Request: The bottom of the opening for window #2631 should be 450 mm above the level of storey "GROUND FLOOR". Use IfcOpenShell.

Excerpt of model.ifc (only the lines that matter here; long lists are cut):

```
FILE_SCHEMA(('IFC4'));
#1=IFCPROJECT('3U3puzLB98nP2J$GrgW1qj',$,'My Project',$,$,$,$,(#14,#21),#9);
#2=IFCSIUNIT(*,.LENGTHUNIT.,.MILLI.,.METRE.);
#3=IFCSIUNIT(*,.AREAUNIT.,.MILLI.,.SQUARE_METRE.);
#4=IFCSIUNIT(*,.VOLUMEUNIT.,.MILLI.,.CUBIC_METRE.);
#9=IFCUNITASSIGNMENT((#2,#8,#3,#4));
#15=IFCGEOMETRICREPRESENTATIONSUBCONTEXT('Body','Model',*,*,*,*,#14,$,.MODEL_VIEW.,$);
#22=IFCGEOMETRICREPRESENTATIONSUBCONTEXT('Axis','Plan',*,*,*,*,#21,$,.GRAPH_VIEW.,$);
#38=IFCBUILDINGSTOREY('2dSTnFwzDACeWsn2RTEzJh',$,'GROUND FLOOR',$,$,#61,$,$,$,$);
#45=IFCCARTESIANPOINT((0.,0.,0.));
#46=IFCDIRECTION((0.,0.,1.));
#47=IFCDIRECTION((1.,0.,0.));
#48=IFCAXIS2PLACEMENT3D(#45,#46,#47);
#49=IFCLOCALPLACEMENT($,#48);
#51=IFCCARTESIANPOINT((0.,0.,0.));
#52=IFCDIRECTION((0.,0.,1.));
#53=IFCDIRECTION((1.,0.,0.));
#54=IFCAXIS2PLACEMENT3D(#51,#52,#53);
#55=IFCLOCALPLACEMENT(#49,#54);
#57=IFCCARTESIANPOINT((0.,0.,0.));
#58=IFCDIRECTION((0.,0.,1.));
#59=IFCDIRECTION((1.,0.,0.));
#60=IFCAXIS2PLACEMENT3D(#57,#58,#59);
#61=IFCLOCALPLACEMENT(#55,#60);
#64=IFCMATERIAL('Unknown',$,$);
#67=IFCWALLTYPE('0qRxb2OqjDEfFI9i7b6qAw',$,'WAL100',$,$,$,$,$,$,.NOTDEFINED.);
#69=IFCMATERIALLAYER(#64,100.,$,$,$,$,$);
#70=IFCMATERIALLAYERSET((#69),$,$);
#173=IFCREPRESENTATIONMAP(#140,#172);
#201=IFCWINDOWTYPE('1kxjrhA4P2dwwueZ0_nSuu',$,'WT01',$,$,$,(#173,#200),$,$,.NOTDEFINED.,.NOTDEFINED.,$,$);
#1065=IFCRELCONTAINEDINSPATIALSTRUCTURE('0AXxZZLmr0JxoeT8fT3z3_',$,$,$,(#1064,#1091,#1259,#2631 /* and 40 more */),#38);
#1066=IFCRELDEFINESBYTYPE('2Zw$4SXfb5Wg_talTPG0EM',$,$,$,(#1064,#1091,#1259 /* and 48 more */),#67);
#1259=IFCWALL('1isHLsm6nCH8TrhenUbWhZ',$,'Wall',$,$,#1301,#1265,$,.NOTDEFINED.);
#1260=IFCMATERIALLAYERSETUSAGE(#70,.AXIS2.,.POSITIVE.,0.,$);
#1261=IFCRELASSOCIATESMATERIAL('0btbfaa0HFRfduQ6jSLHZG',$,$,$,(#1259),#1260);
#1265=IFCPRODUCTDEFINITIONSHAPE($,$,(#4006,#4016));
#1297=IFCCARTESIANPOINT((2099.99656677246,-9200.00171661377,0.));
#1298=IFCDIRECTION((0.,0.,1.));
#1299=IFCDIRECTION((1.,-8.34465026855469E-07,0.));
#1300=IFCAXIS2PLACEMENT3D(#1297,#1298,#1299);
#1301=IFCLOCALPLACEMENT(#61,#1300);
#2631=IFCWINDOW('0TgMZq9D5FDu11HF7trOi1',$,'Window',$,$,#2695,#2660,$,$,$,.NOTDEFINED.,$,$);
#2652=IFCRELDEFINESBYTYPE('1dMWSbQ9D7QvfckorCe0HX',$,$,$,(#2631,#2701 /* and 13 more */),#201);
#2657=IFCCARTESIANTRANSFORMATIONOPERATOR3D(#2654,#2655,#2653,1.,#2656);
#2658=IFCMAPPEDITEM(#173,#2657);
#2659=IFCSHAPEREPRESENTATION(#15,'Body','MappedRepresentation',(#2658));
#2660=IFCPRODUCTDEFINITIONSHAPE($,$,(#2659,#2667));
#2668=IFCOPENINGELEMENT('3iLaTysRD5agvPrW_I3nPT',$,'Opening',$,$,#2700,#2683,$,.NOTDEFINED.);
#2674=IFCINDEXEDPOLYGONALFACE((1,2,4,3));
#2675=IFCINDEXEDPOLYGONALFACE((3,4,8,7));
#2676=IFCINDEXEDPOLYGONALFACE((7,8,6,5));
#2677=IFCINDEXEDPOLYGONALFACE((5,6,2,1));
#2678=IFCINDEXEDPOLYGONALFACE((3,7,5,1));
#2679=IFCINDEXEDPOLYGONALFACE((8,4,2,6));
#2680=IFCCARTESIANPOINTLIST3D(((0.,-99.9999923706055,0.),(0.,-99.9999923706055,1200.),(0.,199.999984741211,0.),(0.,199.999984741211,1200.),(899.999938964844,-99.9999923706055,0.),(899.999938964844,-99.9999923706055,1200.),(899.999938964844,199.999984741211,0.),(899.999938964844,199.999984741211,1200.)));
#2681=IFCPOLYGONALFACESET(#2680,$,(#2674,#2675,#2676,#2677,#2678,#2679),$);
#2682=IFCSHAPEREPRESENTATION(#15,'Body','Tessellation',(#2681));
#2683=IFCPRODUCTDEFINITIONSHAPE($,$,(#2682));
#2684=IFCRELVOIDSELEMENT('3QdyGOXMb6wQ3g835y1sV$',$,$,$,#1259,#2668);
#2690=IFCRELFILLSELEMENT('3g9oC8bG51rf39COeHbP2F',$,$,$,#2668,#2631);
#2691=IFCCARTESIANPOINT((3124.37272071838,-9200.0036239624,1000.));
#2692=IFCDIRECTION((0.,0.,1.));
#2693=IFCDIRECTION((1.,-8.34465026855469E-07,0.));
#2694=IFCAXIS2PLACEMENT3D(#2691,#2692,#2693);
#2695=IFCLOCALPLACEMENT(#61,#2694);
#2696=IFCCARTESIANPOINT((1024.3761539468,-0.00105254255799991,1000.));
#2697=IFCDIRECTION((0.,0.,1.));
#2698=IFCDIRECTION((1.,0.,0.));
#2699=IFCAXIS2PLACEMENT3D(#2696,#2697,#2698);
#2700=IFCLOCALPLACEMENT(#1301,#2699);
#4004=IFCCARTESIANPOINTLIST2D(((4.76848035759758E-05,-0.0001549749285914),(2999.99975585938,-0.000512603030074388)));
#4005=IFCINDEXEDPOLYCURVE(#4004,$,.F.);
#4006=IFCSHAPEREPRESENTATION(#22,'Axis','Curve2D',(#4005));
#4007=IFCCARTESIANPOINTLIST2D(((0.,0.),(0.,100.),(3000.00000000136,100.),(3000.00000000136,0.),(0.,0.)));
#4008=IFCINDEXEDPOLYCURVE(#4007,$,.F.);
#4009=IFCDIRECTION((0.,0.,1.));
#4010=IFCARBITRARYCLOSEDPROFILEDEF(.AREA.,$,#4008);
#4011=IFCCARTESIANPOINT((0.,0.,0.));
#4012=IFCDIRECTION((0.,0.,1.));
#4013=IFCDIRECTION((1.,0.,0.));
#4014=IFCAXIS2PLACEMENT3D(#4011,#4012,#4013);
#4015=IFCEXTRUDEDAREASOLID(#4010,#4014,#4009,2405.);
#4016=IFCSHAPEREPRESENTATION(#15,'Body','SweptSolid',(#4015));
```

```python
import numpy as np
import ifcopenshell
import ifcopenshell.api.geometry
import ifcopenshell.geom
import ifcopenshell.util.element
import ifcopenshell.util.placement
import ifcopenshell.util.shape
import ifcopenshell.util.unit

model = ifcopenshell.open("model.ifc")
unit_scale = ifcopenshell.util.unit.calculate_unit_scale(model)

window = model.by_guid("0TgMZq9D5FDu11HF7trOi1")
opening = window.FillsVoids[0].RelatingOpeningElement
storey = ifcopenshell.util.element.get_container(window, ifc_class="IfcBuildingStorey")
level = ifcopenshell.util.placement.get_local_placement(storey.ObjectPlacement)[2, 3]

# The opening's origin need not be at the sill, so measure its lowest point.
shape = ifcopenshell.geom.create_shape(ifcopenshell.geom.settings(), opening)
bottom = ifcopenshell.util.shape.get_shape_bottom_elevation(shape, shape.geometry) / unit_scale
dz = level + 0.45 / unit_scale - bottom

shift = np.array([0.0, 0.0, dz])
# The window is not placed relative to its opening, so move both.
for product in (opening, window):
    matrix = ifcopenshell.util.placement.get_local_placement(product.ObjectPlacement)
    matrix[:3, 3] += shift
    ifcopenshell.api.geometry.edit_object_placement(model, product=product, matrix=matrix, is_si=False)

print(f"moved by {dz * unit_scale:+.3f} m")

model.write("model_v2.ifc")
```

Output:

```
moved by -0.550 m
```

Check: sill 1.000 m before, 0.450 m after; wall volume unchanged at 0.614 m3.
